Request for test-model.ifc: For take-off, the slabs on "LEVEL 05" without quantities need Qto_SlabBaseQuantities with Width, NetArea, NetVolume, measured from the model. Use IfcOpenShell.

First a look at what the model holds.

```python
import ifcopenshell
import ifcopenshell.util.element
import ifcopenshell.util.unit

model = ifcopenshell.open("test-model.ifc")
print(model.schema)
for unit_type in ("LENGTHUNIT", "AREAUNIT", "VOLUMEUNIT"):
    print(unit_type, ifcopenshell.util.unit.calculate_unit_scale(model, unit_type))
storey = next(s for s in model.by_type("IfcBuildingStorey") if s.Name == "LEVEL 05")
slabs = [e for e in ifcopenshell.util.element.get_decomposition(storey) if e.is_a("IfcSlab")]
for e in sorted(slabs, key=lambda e: e.id()):
    print(e.id(), e.is_a(), e.Name, list(ifcopenshell.util.element.get_psets(e, qtos_only=True)), sep=" | ")
```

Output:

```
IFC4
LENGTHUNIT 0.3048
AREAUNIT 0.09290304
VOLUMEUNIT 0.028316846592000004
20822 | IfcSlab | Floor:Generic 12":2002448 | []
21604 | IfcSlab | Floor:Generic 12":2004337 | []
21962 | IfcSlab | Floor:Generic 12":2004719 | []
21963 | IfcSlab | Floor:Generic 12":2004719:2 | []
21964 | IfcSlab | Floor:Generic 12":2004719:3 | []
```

```python
import ifcopenshell
import ifcopenshell.api.pset
import ifcopenshell.geom
import ifcopenshell.util.element
import ifcopenshell.util.shape
import ifcopenshell.util.unit

model = ifcopenshell.open("test-model.ifc")
unit_scale = ifcopenshell.util.unit.calculate_unit_scale(model)
area_scale = ifcopenshell.util.unit.calculate_unit_scale(model, "AREAUNIT")
volume_scale = ifcopenshell.util.unit.calculate_unit_scale(model, "VOLUMEUNIT")
settings = ifcopenshell.geom.settings()

storey = next(s for s in model.by_type("IfcBuildingStorey") if s.Name == "LEVEL 05")
slabs = [e for e in ifcopenshell.util.element.get_decomposition(storey) if e.is_a("IfcSlab")]

for e in sorted(slabs, key=lambda e: e.id()):
    if ifcopenshell.util.element.get_psets(e, qtos_only=True, should_inherit=False):
        continue
    # Geometry comes back in metres, in the element's own axes.
    shape = ifcopenshell.geom.create_shape(settings, e)
    values = {
        "Width": ifcopenshell.util.shape.get_z(shape.geometry) / unit_scale,
        "NetArea": ifcopenshell.util.shape.get_footprint_area(shape.geometry) / area_scale,
        "NetVolume": ifcopenshell.util.shape.get_volume(shape.geometry) / volume_scale,
    }
    qto = ifcopenshell.api.pset.add_qto(model, product=e, name="Qto_SlabBaseQuantities")
    ifcopenshell.api.pset.edit_qto(model, qto=qto, properties=values)
    print(e.id(), {k: round(v, 3) for k, v in values.items()})

model.write("test-model_updated.ifc")
```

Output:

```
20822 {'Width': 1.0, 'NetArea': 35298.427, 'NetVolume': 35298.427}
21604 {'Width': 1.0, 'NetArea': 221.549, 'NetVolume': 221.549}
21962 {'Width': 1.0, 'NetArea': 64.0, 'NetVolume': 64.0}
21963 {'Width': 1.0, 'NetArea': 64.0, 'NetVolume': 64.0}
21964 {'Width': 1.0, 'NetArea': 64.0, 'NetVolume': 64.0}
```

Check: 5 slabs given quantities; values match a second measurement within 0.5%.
